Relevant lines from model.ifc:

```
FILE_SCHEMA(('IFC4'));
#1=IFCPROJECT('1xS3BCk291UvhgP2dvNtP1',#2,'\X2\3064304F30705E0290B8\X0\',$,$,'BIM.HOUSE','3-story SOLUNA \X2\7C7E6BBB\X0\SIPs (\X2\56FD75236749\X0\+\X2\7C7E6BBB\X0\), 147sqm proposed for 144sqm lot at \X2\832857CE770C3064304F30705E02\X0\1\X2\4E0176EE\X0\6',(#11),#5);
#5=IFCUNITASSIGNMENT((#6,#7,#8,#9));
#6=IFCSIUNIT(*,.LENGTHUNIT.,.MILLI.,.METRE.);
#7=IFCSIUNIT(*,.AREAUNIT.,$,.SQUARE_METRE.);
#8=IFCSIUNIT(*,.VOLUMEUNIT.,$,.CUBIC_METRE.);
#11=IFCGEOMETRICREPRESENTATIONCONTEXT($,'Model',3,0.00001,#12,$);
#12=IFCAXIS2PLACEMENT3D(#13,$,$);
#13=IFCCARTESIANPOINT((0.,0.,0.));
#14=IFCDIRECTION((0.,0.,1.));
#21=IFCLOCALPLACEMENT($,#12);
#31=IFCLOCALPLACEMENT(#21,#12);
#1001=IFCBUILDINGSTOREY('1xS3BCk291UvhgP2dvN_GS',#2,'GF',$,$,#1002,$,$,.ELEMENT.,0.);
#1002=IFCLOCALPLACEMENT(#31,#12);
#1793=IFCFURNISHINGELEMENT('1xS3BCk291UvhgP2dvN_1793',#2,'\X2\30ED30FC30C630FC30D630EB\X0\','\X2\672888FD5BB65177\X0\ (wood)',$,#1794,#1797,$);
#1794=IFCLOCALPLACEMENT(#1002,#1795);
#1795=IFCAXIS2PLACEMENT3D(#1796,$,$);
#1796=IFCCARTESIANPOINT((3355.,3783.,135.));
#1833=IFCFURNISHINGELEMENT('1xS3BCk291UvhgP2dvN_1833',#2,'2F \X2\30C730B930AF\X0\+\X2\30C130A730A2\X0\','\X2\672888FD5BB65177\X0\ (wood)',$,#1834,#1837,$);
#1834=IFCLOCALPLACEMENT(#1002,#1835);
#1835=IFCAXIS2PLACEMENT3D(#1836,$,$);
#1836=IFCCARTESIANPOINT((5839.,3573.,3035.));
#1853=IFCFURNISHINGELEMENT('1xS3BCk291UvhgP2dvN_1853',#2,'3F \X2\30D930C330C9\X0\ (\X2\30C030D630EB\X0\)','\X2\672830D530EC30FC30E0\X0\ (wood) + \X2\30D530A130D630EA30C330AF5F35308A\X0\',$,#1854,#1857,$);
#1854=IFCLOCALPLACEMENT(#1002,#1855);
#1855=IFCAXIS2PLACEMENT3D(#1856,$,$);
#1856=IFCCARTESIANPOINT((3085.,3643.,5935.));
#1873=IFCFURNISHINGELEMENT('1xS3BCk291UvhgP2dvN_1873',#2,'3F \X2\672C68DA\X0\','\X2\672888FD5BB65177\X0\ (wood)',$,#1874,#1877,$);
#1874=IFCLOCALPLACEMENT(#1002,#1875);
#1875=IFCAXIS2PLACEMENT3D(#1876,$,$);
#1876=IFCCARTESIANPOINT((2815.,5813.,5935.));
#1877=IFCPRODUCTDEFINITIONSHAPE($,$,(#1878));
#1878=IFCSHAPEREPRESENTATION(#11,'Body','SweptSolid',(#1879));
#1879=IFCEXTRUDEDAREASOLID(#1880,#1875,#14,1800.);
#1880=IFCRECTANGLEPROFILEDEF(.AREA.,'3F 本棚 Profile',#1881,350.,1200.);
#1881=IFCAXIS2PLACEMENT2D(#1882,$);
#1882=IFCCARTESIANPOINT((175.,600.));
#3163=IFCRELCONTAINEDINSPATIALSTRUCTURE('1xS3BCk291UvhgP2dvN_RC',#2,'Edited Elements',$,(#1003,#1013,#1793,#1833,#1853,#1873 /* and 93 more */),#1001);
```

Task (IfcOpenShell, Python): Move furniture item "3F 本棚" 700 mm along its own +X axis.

```python
import ifcopenshell
import ifcopenshell.api.geometry
import ifcopenshell.util.placement
import ifcopenshell.util.unit

model = ifcopenshell.open("model.ifc")
unit_scale = ifcopenshell.util.unit.calculate_unit_scale(model)

item = model.by_guid("1xS3BCk291UvhgP2dvN_1873")
matrix = ifcopenshell.util.placement.get_local_placement(item.ObjectPlacement)
matrix[:3, 3] += matrix[:3, 0] * 0.7 / unit_scale
ifcopenshell.api.geometry.edit_object_placement(model, product=item, matrix=matrix, is_si=False)

print(ifcopenshell.util.placement.get_local_placement(item.ObjectPlacement).round(3) + 0.0)

model.write("model_rev.ifc")
```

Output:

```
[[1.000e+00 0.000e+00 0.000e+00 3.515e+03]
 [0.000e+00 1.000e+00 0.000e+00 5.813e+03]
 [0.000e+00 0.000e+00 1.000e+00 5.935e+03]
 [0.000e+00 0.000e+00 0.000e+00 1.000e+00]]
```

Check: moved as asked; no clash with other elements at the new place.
